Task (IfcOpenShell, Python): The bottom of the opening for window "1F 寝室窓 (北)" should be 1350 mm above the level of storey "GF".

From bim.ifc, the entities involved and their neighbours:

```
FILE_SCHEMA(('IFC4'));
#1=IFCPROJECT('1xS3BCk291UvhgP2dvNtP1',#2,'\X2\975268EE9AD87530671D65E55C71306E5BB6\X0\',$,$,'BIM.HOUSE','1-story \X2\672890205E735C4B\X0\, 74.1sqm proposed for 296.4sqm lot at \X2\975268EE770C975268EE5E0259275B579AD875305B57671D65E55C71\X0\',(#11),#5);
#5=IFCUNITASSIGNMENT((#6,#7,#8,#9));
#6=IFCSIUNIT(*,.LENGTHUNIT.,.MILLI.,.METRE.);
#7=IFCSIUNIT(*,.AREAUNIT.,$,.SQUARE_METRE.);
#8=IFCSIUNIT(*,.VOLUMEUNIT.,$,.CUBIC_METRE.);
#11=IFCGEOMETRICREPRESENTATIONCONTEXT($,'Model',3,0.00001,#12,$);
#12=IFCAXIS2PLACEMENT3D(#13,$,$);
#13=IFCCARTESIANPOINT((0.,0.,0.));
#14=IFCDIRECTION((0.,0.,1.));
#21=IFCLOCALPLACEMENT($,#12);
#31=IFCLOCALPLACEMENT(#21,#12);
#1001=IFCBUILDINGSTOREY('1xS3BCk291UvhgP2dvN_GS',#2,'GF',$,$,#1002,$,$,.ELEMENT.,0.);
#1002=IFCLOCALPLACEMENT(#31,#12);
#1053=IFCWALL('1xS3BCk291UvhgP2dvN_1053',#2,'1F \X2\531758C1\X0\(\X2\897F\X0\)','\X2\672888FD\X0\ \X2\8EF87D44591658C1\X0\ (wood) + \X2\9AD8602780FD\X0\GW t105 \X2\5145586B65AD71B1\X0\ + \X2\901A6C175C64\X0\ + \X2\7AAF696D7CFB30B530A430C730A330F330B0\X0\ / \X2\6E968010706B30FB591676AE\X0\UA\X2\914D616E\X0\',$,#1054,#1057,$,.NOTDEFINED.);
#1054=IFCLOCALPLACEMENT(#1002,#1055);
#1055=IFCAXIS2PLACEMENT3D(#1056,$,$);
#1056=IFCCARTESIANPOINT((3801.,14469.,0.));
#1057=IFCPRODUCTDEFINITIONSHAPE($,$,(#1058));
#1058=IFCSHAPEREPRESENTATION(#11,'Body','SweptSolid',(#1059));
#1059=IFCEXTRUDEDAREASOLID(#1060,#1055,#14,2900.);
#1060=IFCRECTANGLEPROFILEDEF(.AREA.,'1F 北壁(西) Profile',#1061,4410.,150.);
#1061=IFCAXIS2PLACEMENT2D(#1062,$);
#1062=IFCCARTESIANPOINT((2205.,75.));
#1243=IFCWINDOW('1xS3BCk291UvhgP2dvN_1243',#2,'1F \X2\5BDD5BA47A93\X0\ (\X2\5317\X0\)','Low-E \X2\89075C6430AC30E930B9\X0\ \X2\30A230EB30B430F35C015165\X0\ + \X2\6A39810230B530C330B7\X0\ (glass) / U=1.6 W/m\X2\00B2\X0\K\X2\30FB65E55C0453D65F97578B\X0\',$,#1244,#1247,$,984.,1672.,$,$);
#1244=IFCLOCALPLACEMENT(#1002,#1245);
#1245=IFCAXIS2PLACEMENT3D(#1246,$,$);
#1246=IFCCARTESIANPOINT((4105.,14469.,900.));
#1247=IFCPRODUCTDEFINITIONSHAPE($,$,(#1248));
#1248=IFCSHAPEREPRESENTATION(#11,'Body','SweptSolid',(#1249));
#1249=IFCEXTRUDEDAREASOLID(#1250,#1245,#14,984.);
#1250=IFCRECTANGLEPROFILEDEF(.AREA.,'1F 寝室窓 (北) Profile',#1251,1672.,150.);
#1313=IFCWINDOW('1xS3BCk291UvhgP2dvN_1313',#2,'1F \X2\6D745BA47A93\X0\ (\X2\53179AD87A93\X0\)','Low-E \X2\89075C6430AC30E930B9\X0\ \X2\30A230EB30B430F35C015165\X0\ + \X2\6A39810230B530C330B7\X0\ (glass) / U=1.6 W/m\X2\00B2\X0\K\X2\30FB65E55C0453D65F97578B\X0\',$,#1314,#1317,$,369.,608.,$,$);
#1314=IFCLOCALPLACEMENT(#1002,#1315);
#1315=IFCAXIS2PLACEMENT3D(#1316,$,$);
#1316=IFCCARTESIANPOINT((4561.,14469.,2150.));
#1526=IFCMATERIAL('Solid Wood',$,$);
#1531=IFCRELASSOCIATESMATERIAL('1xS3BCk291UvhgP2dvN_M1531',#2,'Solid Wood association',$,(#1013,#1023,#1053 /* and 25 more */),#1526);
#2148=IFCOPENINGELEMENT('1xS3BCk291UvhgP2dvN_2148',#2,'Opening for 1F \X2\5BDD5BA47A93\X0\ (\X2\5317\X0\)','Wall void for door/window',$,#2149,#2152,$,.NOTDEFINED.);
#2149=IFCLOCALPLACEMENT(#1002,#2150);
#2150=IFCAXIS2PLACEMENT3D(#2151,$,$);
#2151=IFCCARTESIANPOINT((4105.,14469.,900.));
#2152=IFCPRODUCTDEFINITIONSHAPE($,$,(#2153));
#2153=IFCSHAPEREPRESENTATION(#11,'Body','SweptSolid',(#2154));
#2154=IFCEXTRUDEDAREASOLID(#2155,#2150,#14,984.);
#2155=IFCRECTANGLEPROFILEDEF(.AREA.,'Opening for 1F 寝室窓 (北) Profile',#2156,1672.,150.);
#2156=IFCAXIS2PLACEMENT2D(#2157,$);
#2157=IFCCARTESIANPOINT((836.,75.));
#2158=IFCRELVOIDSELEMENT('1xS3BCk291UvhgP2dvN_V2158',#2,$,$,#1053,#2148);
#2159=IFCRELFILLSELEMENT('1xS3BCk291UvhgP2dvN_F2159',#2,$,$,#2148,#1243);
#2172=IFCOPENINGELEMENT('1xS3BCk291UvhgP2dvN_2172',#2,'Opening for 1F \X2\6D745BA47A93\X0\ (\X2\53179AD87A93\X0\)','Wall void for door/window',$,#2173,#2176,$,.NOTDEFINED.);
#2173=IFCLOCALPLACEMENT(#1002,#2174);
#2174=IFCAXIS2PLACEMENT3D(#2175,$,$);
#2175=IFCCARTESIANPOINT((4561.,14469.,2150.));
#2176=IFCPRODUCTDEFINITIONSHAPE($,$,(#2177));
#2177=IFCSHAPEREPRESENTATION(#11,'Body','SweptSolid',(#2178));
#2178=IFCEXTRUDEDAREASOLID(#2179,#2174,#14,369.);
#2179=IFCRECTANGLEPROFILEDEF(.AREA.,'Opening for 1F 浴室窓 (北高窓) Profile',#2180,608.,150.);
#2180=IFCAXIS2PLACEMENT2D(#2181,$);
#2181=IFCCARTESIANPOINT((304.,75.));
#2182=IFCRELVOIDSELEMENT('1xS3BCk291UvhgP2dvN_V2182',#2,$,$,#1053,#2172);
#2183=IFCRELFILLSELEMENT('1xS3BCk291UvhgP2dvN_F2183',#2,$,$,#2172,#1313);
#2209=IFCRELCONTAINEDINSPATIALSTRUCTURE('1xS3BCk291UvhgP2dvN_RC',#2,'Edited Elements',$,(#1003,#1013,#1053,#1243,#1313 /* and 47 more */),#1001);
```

```python
import numpy as np
import ifcopenshell
import ifcopenshell.api.geometry
import ifcopenshell.geom
import ifcopenshell.util.element
import ifcopenshell.util.placement
import ifcopenshell.util.shape
import ifcopenshell.util.unit

model = ifcopenshell.open("bim.ifc")
unit_scale = ifcopenshell.util.unit.calculate_unit_scale(model)

window = model.by_id(1243)
opening = window.FillsVoids[0].RelatingOpeningElement
storey = ifcopenshell.util.element.get_container(window, ifc_class="IfcBuildingStorey")
level = ifcopenshell.util.placement.get_local_placement(storey.ObjectPlacement)[2, 3]

# The opening's origin need not be at the sill, so measure its lowest point.
shape = ifcopenshell.geom.create_shape(ifcopenshell.geom.settings(), opening)
bottom = ifcopenshell.util.shape.get_shape_bottom_elevation(shape, shape.geometry) / unit_scale
dz = level + 1.35 / unit_scale - bottom

shift = np.array([0.0, 0.0, dz])
# The window is not placed relative to its opening, so move both.
for product in (opening, window):
    matrix = ifcopenshell.util.placement.get_local_placement(product.ObjectPlacement)
    matrix[:3, 3] += shift
    ifcopenshell.api.geometry.edit_object_placement(model, product=product, matrix=matrix, is_si=False)

print(f"moved by {dz * unit_scale:+.3f} m")

model.write("bim_edited.ifc")
```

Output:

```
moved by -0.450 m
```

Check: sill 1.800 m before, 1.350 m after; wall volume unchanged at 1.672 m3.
